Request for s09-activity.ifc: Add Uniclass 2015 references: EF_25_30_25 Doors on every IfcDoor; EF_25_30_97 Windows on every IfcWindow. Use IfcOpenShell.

First a look at what the model holds.

```python
import ifcopenshell

model = ifcopenshell.open("s09-activity.ifc")
print(model.schema)
print("classifications:", [c.Name for c in model.by_type("IfcClassification")])
for ifc_class in ("IfcDoor", "IfcRoof", "IfcStair", "IfcWall", "IfcWindow"):
    print(ifc_class, len(model.by_type(ifc_class)))
```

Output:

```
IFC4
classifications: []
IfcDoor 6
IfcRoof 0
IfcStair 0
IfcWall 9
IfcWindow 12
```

```python
import ifcopenshell
import ifcopenshell.api.classification

model = ifcopenshell.open("s09-activity.ifc")

system = ifcopenshell.api.classification.add_classification(model, classification="Uniclass 2015")

codes = {
    "IfcDoor": ("EF_25_30_25", "Doors"),
    "IfcWindow": ("EF_25_30_97", "Windows"),
}
for ifc_class, (code, name) in codes.items():
    products = model.by_type(ifc_class)
    ifcopenshell.api.classification.add_reference(
        model, products=products, classification=system, identification=code, name=name
    )
    print(code, len(products))

model.write("s09-activity-out.ifc")
```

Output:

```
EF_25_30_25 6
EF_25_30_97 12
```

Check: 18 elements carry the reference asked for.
